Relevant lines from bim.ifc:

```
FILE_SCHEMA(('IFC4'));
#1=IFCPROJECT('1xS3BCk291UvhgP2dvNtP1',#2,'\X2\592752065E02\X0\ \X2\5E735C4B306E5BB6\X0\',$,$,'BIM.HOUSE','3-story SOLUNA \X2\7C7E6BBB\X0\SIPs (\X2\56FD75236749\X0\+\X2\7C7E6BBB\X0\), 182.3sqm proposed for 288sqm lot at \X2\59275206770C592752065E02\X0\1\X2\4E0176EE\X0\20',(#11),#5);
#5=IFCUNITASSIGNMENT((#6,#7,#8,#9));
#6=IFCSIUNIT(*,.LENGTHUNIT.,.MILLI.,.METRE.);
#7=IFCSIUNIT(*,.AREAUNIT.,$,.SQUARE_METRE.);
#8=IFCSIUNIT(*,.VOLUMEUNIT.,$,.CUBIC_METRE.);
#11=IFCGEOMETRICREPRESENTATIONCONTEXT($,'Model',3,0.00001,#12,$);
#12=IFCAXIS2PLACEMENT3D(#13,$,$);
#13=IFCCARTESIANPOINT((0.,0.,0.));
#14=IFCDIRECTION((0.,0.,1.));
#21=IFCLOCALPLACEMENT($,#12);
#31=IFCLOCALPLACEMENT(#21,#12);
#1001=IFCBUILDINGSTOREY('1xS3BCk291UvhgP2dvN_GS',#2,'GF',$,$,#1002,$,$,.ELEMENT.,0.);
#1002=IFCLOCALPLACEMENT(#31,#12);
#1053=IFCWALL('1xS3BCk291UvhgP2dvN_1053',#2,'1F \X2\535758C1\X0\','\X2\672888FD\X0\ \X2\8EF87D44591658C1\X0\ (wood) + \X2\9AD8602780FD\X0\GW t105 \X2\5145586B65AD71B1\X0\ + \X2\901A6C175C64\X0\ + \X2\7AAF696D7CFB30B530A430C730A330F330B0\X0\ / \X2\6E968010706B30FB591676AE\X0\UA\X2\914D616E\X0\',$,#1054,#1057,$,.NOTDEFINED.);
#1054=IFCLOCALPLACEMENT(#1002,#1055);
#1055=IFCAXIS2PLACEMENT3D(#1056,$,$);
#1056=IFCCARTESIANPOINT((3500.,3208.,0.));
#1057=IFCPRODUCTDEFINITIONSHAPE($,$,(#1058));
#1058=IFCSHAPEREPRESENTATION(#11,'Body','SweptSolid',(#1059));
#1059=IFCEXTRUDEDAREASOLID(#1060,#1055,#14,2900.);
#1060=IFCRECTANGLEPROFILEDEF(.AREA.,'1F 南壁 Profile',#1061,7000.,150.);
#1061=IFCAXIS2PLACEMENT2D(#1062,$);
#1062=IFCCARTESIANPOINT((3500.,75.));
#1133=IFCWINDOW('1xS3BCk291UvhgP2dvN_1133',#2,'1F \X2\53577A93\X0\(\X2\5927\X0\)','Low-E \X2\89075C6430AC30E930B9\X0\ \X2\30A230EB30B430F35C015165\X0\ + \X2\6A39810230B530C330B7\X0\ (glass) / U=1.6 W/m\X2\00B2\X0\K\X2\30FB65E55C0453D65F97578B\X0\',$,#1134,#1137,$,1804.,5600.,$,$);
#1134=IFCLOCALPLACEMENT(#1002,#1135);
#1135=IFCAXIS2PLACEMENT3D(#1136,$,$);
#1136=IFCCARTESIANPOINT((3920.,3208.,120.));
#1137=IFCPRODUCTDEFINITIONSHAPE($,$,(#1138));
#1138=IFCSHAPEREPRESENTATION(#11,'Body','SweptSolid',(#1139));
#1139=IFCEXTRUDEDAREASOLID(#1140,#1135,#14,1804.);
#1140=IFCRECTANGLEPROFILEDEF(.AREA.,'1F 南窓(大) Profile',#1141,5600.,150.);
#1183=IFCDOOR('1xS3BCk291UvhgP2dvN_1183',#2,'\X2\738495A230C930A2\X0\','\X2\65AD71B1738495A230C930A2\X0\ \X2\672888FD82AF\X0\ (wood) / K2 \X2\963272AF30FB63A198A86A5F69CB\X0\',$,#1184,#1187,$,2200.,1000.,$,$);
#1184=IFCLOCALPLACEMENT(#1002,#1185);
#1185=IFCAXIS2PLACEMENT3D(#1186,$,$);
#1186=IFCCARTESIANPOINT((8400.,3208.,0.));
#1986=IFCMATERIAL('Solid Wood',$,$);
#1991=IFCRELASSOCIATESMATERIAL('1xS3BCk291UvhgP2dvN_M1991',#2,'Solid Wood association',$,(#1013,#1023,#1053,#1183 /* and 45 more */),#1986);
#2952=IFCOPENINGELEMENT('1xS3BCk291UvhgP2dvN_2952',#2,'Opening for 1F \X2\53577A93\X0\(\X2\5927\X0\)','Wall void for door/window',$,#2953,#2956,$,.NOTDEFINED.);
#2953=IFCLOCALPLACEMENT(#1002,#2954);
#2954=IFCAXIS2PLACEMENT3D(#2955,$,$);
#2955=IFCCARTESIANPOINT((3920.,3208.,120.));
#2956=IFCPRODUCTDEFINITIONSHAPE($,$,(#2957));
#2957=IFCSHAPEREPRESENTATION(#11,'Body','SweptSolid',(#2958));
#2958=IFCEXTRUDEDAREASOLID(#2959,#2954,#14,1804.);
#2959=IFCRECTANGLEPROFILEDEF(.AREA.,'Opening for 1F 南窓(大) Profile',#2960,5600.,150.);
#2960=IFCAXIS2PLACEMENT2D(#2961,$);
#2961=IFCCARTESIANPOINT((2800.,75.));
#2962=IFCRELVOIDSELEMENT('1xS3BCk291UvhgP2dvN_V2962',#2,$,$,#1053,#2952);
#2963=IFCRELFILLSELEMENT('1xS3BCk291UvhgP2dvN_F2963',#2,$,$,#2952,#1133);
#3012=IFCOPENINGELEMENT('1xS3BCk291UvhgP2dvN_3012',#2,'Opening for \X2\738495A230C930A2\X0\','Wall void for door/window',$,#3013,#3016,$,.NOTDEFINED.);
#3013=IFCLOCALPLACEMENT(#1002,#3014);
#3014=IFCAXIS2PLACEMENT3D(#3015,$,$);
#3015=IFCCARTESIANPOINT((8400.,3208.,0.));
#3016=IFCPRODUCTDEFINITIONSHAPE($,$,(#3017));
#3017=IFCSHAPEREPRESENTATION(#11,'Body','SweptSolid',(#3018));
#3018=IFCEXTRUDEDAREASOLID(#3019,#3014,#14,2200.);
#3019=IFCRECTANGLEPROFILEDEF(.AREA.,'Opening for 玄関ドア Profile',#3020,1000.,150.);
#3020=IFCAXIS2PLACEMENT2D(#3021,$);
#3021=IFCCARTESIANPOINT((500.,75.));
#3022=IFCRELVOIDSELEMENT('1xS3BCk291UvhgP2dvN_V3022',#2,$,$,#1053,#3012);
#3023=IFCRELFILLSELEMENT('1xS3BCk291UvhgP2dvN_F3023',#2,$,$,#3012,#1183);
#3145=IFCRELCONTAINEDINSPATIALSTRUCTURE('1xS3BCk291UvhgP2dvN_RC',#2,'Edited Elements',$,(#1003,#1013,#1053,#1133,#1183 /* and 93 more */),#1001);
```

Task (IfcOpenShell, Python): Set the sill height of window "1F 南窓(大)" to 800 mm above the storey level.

```python
import numpy as np
import ifcopenshell
import ifcopenshell.api.geometry
import ifcopenshell.geom
import ifcopenshell.util.element
import ifcopenshell.util.placement
import ifcopenshell.util.shape
import ifcopenshell.util.unit

model = ifcopenshell.open("bim.ifc")
unit_scale = ifcopenshell.util.unit.calculate_unit_scale(model)

window = model.by_guid("1xS3BCk291UvhgP2dvN_1133")
opening = window.FillsVoids[0].RelatingOpeningElement
storey = ifcopenshell.util.element.get_container(window, ifc_class="IfcBuildingStorey")
level = ifcopenshell.util.placement.get_local_placement(storey.ObjectPlacement)[2, 3]

# The opening's origin need not be at the sill, so measure its lowest point.
shape = ifcopenshell.geom.create_shape(ifcopenshell.geom.settings(), opening)
bottom = ifcopenshell.util.shape.get_shape_bottom_elevation(shape, shape.geometry) / unit_scale
dz = level + 800.0 - bottom

shift = np.array([0.0, 0.0, dz])
# The window is not placed relative to its opening, so move both.
for product in (opening, window):
    matrix = ifcopenshell.util.placement.get_local_placement(product.ObjectPlacement)
    matrix[:3, 3] += shift
    ifcopenshell.api.geometry.edit_object_placement(model, product=product, matrix=matrix, is_si=False)

print(f"moved by {dz * unit_scale:+.3f} m")

model.write("bim-out.ifc")
```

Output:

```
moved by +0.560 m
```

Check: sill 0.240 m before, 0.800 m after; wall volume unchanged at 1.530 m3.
